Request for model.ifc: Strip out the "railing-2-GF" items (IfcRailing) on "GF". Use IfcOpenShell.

First a look at what the model holds.

```python
import ifcopenshell
import ifcopenshell.util.element

model = ifcopenshell.open("model.ifc")
print(model.schema)
storey = next(s for s in model.by_type("IfcBuildingStorey") if s.Name == "GF")
railings = [e for e in ifcopenshell.util.element.get_decomposition(storey) if e.is_a("IfcRailing")]
seen = {}
for e in railings:
    element_type = ifcopenshell.util.element.get_type(e)
    name = element_type.Name if element_type not in (None, e) else None
    seen[name] = seen.get(name, 0) + 1
for name, count in sorted(seen.items(), key=str):
    print(count, "x", name)
```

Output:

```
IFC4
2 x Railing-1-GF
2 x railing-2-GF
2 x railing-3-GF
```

```python
import ifcopenshell
import ifcopenshell.api.root
import ifcopenshell.util.element

model = ifcopenshell.open("model.ifc")

storey = next(s for s in model.by_type("IfcBuildingStorey") if s.Name == "GF")
railings = [e for e in ifcopenshell.util.element.get_decomposition(storey) if e.is_a("IfcRailing")]
targets = [e for e in railings if (t := ifcopenshell.util.element.get_type(e)) not in (None, e) and t.Name == "railing-2-GF"]

for e in targets:
    ifcopenshell.api.root.remove_product(model, product=e)
print(len(targets), "removed")

model.write("model_edited.ifc")
```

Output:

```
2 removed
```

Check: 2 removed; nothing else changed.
